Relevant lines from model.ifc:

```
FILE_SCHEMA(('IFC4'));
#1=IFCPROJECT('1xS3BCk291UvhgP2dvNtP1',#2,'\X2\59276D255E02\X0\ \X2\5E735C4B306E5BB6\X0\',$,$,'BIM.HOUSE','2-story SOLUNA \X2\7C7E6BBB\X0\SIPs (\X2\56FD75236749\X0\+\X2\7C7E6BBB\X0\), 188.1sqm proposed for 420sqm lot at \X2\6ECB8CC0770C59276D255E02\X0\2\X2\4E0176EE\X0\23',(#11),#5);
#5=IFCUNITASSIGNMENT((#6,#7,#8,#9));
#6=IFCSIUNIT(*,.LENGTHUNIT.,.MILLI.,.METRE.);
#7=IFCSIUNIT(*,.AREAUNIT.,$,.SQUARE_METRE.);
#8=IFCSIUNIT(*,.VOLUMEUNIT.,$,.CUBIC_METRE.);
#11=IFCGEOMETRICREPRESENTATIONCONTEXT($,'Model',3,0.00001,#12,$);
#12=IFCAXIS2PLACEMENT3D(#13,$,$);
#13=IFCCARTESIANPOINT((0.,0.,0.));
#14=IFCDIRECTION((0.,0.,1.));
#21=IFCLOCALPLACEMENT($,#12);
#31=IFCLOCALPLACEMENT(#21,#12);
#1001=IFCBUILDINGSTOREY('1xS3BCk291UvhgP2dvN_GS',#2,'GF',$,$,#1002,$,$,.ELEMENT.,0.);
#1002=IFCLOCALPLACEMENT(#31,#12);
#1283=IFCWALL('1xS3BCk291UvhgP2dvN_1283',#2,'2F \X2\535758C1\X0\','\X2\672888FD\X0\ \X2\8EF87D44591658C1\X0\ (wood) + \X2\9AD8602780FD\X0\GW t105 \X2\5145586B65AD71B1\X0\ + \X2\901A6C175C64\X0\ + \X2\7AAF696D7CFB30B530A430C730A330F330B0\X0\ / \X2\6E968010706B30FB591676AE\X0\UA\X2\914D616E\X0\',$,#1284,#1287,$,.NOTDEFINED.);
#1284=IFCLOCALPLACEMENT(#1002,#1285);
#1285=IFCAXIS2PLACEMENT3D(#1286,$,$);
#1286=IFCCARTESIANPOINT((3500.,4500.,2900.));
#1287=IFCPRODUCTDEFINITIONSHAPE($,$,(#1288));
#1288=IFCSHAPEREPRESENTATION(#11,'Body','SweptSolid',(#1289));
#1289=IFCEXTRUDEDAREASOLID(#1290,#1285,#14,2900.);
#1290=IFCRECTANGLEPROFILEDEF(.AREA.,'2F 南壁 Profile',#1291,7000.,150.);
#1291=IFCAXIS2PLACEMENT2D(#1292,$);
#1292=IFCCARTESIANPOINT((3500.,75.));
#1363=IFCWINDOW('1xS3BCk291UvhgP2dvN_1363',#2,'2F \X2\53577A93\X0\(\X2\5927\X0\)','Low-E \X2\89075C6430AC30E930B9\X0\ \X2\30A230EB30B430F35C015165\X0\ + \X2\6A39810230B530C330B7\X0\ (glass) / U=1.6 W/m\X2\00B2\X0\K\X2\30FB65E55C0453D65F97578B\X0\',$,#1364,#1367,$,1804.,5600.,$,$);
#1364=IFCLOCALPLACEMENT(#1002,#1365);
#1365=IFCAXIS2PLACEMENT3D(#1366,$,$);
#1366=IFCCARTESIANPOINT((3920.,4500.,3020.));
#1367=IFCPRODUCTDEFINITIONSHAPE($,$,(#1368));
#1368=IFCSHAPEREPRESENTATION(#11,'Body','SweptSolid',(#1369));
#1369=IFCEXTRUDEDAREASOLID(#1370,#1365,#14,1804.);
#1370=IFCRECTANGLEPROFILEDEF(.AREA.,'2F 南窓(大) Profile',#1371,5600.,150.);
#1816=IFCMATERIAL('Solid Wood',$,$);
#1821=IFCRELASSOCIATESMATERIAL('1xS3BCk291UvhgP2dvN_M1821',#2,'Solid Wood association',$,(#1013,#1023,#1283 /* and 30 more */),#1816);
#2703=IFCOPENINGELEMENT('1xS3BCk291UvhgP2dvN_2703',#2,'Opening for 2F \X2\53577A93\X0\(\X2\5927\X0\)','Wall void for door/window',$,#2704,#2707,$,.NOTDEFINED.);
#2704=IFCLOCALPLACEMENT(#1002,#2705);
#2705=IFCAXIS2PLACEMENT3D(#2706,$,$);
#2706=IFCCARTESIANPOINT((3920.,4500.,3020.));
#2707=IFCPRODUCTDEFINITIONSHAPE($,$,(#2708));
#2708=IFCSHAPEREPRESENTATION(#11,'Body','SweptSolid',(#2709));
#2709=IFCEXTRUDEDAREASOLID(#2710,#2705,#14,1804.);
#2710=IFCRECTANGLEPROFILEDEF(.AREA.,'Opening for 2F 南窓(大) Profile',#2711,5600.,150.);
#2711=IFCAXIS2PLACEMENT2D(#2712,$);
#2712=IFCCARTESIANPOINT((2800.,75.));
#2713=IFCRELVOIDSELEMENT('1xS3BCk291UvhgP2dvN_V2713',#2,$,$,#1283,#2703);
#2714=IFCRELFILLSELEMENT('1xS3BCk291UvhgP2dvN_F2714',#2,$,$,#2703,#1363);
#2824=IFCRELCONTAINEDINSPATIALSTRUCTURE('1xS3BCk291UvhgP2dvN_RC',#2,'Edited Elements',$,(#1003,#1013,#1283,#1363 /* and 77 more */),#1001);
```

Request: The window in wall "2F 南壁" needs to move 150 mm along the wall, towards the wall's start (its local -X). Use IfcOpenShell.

```python
import ifcopenshell
import ifcopenshell.api.geometry
import ifcopenshell.util.placement

model = ifcopenshell.open("model.ifc")

window = model.by_guid("1xS3BCk291UvhgP2dvN_1363")
opening = window.FillsVoids[0].RelatingOpeningElement
wall = opening.VoidsElements[0].RelatingBuildingElement

wall_matrix = ifcopenshell.util.placement.get_local_placement(wall.ObjectPlacement)
shift = wall_matrix[:3, 0] * -150.0
before = ifcopenshell.util.placement.get_local_placement(window.ObjectPlacement)[:3, 3].copy()

# The window is not placed relative to its opening, so move both.
for product in (opening, window):
    matrix = ifcopenshell.util.placement.get_local_placement(product.ObjectPlacement)
    matrix[:3, 3] += shift
    ifcopenshell.api.geometry.edit_object_placement(model, product=product, matrix=matrix, is_si=False)

after = ifcopenshell.util.placement.get_local_placement(window.ObjectPlacement)[:3, 3]
print("window moved by", (after - before).round(3) + 0.0)

model.write("model-out.ifc")
```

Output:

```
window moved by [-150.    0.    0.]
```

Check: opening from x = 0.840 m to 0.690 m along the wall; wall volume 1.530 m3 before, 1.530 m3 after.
